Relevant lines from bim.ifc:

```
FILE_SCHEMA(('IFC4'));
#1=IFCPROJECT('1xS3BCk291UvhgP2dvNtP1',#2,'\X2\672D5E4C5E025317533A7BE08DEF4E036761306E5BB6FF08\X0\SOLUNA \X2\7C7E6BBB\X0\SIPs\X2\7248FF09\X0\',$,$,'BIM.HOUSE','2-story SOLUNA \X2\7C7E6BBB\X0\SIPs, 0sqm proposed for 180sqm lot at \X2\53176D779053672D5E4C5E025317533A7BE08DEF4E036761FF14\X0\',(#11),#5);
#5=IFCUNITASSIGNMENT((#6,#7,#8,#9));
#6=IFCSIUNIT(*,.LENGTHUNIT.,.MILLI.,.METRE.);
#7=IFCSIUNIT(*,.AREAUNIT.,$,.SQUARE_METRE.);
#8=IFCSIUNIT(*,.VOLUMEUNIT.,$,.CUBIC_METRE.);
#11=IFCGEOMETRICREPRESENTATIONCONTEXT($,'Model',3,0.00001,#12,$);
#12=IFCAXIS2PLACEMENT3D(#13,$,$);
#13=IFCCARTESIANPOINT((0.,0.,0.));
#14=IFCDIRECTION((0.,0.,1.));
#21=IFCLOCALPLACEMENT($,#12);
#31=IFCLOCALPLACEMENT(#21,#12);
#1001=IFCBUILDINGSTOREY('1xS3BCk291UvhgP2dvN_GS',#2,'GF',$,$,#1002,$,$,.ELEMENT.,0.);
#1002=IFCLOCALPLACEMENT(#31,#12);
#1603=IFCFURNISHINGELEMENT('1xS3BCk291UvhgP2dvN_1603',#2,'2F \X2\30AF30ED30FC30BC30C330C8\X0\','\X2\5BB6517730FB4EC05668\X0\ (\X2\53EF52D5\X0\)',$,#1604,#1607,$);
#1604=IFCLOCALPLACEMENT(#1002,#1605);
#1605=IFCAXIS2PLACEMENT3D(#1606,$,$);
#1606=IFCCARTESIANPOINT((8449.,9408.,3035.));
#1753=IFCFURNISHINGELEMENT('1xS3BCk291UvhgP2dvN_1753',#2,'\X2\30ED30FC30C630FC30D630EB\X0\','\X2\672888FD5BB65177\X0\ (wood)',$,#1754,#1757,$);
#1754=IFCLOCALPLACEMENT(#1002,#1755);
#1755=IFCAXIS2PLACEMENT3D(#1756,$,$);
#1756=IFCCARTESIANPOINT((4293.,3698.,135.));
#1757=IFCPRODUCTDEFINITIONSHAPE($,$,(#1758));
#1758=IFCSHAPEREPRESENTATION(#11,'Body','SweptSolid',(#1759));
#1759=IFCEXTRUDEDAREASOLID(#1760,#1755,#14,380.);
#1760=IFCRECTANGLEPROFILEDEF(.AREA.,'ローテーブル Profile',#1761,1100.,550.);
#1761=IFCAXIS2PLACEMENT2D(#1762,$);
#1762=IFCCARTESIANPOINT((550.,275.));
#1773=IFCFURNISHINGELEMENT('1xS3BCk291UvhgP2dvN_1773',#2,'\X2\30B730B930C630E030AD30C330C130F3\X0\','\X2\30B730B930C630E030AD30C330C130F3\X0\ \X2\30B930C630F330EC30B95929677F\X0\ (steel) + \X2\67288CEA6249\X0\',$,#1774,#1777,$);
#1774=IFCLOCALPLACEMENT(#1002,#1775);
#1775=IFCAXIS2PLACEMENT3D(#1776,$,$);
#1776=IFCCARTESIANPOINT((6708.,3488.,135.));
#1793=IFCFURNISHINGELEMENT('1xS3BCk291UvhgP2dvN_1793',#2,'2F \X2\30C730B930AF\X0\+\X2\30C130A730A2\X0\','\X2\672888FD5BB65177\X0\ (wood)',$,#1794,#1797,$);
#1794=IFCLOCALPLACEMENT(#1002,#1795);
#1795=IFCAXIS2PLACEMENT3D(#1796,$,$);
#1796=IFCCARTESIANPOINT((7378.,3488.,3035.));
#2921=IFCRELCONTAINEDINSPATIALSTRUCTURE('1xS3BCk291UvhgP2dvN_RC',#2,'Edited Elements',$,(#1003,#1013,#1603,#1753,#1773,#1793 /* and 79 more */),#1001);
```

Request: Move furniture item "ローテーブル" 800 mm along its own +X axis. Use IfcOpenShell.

```python
import ifcopenshell
import ifcopenshell.api.geometry
import ifcopenshell.util.placement
import ifcopenshell.util.unit

model = ifcopenshell.open("bim.ifc")
unit_scale = ifcopenshell.util.unit.calculate_unit_scale(model)

item = model.by_guid("1xS3BCk291UvhgP2dvN_1753")
matrix = ifcopenshell.util.placement.get_local_placement(item.ObjectPlacement)
matrix[:3, 3] += matrix[:3, 0] * 0.8 / unit_scale
ifcopenshell.api.geometry.edit_object_placement(model, product=item, matrix=matrix, is_si=False)

print(ifcopenshell.util.placement.get_local_placement(item.ObjectPlacement).round(3) + 0.0)

model.write("bim-out.ifc")
```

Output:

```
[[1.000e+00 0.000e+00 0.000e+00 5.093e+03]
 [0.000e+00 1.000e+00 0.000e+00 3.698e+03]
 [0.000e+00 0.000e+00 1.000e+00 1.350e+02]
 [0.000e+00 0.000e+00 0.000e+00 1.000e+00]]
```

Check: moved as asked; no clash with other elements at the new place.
